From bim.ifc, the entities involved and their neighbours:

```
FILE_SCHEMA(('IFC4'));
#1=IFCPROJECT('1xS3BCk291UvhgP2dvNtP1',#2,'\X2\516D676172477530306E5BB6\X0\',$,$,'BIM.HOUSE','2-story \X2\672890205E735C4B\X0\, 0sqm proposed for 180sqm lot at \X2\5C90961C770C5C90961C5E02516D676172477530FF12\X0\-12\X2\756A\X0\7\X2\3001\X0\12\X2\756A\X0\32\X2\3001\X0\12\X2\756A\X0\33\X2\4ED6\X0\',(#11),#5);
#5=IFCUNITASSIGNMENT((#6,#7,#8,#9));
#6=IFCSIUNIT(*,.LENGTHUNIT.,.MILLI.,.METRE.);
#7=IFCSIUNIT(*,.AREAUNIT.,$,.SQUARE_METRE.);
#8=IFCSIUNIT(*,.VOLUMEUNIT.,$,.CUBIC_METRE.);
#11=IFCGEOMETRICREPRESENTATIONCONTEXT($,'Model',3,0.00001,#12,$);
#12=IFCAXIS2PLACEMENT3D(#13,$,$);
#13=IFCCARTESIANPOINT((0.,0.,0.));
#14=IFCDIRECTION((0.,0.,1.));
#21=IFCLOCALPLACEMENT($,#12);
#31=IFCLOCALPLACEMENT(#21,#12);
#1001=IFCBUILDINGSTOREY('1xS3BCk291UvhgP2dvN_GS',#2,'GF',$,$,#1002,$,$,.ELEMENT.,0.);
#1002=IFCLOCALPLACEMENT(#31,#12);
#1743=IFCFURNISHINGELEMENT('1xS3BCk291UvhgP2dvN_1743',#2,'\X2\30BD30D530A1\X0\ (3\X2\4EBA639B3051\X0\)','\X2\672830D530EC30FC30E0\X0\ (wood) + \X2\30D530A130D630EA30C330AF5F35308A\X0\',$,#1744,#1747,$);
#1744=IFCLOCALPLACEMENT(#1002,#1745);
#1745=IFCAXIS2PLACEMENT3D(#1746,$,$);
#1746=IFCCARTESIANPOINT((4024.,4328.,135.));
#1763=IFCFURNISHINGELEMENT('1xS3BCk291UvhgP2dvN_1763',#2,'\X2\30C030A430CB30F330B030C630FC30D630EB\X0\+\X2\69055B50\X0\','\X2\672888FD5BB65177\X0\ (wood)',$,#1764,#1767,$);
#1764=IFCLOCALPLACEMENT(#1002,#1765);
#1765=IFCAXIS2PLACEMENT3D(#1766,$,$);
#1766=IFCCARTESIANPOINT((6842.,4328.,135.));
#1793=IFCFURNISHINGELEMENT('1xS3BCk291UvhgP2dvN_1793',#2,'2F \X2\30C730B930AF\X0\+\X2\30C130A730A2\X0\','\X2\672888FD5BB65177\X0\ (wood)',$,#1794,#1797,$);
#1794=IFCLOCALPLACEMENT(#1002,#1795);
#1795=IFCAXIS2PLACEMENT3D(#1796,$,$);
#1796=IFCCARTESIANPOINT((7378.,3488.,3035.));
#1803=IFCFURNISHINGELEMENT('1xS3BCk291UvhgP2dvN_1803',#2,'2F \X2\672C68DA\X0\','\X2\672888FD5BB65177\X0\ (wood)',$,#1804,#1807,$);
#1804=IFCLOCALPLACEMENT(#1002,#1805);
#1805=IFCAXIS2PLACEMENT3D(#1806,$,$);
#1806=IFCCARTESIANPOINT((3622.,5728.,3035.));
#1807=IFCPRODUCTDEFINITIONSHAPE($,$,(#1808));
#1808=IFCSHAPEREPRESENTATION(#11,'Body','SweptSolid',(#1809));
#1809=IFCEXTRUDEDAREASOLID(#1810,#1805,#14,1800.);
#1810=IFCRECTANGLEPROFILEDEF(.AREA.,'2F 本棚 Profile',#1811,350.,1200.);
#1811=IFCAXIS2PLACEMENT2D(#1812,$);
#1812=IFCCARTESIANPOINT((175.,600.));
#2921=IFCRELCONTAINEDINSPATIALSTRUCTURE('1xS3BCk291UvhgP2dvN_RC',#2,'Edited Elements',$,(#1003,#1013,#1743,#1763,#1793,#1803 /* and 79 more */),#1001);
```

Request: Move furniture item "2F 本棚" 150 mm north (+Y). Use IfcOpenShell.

```python
import ifcopenshell
import ifcopenshell.api.geometry
import ifcopenshell.util.placement
import ifcopenshell.util.unit

model = ifcopenshell.open("bim.ifc")
unit_scale = ifcopenshell.util.unit.calculate_unit_scale(model)

item = model.by_guid("1xS3BCk291UvhgP2dvN_1803")
matrix = ifcopenshell.util.placement.get_local_placement(item.ObjectPlacement)
matrix[1, 3] += 0.15 / unit_scale
ifcopenshell.api.geometry.edit_object_placement(model, product=item, matrix=matrix, is_si=False)

print(ifcopenshell.util.placement.get_local_placement(item.ObjectPlacement).round(3) + 0.0)

model.write("bim_edited.ifc")
```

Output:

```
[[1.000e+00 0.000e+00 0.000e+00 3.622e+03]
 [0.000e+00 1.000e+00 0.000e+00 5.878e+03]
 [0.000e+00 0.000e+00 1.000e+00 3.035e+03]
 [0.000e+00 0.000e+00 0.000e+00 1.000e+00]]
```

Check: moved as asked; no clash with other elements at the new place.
